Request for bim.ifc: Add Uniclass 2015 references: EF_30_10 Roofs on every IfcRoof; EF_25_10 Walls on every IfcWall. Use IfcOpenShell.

First a look at what the model holds.

```python
import ifcopenshell

model = ifcopenshell.open("bim.ifc")
print(model.schema)
print("classifications:", [c.Name for c in model.by_type("IfcClassification")])
for ifc_class in ("IfcDoor", "IfcRoof", "IfcStair", "IfcWall", "IfcWindow"):
    print(ifc_class, len(model.by_type(ifc_class)))
```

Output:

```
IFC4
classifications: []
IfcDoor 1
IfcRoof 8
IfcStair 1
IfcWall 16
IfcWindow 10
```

```python
import ifcopenshell
import ifcopenshell.api.classification

model = ifcopenshell.open("bim.ifc")

system = ifcopenshell.api.classification.add_classification(model, classification="Uniclass 2015")

codes = {
    "IfcRoof": ("EF_30_10", "Roofs"),
    "IfcWall": ("EF_25_10", "Walls"),
}
for ifc_class, (code, name) in codes.items():
    products = model.by_type(ifc_class)
    ifcopenshell.api.classification.add_reference(
        model, products=products, classification=system, identification=code, name=name
    )
    print(code, len(products))

model.write("bim_rev.ifc")
```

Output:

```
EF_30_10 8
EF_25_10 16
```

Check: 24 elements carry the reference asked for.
